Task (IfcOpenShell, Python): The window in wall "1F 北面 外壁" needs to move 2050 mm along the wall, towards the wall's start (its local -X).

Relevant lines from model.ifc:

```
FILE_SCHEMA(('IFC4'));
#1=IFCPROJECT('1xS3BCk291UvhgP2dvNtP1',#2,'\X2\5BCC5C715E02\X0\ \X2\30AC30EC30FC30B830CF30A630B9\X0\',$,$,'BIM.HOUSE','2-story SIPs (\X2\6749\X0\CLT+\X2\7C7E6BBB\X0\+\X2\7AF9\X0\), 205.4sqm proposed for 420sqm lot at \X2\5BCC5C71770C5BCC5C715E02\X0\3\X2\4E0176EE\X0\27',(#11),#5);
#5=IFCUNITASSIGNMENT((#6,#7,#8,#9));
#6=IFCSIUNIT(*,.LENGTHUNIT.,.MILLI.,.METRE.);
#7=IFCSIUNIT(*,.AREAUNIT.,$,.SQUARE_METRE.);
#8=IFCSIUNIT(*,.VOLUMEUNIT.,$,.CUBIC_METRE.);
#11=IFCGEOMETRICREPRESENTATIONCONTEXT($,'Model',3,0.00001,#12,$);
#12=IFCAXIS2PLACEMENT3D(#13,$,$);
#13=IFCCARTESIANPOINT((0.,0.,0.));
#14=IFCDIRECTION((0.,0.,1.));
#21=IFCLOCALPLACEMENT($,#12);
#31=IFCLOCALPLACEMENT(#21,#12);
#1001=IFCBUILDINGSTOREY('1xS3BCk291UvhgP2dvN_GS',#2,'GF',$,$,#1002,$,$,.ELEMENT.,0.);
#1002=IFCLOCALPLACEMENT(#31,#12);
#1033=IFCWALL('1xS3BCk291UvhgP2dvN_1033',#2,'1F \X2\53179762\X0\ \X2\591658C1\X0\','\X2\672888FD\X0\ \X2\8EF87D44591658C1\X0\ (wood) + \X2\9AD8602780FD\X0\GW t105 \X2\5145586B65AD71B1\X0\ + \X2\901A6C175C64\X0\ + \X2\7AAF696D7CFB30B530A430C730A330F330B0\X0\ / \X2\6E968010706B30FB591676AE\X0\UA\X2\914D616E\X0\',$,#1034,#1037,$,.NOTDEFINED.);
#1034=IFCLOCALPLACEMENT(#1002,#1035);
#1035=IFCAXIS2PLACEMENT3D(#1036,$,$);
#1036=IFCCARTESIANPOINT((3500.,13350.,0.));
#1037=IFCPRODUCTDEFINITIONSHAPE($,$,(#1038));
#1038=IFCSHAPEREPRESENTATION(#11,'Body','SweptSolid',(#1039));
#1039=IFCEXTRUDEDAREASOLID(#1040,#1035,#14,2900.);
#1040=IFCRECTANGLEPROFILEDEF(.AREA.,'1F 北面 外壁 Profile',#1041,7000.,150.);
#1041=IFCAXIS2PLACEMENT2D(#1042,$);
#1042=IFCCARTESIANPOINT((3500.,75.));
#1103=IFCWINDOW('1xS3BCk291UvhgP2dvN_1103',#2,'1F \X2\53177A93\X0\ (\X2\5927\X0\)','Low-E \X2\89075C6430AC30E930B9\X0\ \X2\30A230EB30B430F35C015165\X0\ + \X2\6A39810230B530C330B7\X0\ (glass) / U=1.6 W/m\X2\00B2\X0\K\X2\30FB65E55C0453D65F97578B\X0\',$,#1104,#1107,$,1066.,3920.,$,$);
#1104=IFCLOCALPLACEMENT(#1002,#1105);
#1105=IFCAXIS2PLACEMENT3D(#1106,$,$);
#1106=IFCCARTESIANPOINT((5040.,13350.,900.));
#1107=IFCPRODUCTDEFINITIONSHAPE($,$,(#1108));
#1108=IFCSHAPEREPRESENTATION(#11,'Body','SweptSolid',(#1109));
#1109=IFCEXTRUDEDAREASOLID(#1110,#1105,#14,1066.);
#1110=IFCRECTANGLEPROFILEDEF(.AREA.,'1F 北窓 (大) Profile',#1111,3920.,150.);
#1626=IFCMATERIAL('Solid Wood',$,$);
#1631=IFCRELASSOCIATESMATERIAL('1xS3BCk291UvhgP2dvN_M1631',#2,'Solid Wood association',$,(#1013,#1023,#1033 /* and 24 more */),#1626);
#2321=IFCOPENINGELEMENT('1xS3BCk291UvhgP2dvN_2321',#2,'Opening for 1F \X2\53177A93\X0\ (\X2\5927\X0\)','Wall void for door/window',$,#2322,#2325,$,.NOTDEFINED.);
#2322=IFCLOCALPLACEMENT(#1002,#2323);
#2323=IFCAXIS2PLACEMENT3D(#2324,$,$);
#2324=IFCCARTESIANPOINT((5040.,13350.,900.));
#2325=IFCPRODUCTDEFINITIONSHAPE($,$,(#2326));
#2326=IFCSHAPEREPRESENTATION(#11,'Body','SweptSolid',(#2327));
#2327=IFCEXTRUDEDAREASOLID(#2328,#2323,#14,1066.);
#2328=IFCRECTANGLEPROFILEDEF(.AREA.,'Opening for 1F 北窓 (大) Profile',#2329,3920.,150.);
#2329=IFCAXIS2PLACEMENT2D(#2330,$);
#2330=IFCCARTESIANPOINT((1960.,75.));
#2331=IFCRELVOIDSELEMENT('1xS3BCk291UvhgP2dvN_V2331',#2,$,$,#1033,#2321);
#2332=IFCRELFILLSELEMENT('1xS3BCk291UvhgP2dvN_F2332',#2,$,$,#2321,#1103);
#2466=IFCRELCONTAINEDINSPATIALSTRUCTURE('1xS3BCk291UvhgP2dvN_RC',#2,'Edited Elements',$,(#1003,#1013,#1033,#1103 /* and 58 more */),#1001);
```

```python
import ifcopenshell
import ifcopenshell.api.geometry
import ifcopenshell.util.placement
import ifcopenshell.util.unit

model = ifcopenshell.open("model.ifc")
unit_scale = ifcopenshell.util.unit.calculate_unit_scale(model)

window = model.by_guid("1xS3BCk291UvhgP2dvN_1103")
opening = window.FillsVoids[0].RelatingOpeningElement
wall = opening.VoidsElements[0].RelatingBuildingElement

wall_matrix = ifcopenshell.util.placement.get_local_placement(wall.ObjectPlacement)
shift = wall_matrix[:3, 0] * -2.05 / unit_scale
before = ifcopenshell.util.placement.get_local_placement(window.ObjectPlacement)[:3, 3].copy()

# The window is not placed relative to its opening, so move both.
for product in (opening, window):
    matrix = ifcopenshell.util.placement.get_local_placement(product.ObjectPlacement)
    matrix[:3, 3] += shift
    ifcopenshell.api.geometry.edit_object_placement(model, product=product, matrix=matrix, is_si=False)

after = ifcopenshell.util.placement.get_local_placement(window.ObjectPlacement)[:3, 3]
print("window moved by", (after - before).round(3) + 0.0)

model.write("model_v2.ifc")
```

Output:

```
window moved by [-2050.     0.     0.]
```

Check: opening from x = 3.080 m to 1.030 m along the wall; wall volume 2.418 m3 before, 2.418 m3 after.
